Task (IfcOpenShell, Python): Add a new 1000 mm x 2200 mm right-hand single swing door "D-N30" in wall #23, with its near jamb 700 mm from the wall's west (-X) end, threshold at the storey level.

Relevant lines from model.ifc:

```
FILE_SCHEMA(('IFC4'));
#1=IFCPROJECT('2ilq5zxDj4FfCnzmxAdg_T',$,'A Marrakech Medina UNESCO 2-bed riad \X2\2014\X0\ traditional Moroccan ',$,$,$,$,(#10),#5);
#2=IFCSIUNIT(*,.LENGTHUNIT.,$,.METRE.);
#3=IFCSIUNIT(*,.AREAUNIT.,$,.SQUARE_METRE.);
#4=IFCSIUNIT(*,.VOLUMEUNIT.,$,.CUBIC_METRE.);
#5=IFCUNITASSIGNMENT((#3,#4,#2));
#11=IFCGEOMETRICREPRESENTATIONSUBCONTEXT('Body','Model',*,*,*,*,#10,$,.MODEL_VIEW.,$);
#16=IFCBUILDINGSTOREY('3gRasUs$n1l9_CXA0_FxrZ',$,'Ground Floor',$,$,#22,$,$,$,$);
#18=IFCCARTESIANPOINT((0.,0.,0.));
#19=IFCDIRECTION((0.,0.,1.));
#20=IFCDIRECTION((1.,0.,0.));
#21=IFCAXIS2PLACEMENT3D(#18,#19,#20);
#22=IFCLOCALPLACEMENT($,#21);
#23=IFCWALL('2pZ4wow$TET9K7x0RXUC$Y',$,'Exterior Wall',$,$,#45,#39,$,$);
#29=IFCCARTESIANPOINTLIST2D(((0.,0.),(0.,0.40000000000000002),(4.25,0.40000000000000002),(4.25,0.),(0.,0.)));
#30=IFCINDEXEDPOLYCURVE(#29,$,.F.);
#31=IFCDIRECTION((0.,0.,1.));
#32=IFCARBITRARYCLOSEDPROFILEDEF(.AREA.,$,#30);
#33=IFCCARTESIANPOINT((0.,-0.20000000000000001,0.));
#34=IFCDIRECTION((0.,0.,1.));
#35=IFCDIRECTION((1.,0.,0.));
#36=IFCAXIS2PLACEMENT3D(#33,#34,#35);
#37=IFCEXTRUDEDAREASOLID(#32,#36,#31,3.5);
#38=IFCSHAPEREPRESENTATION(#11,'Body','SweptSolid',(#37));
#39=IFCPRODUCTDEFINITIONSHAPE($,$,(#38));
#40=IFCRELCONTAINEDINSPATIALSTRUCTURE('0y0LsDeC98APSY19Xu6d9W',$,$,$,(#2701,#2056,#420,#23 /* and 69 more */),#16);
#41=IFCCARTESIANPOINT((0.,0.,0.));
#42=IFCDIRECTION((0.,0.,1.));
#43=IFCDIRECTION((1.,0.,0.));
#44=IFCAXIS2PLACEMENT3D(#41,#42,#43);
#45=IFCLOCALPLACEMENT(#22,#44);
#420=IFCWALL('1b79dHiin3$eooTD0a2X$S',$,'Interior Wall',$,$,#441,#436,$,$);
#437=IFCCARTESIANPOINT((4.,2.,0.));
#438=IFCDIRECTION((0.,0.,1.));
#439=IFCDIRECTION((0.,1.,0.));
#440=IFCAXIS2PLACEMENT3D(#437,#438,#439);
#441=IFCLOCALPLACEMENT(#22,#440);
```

```python
import numpy as np
import ifcopenshell
import ifcopenshell.api.feature
import ifcopenshell.api.geometry
import ifcopenshell.api.root
import ifcopenshell.api.spatial
import ifcopenshell.geom
import ifcopenshell.util.element
import ifcopenshell.util.placement
import ifcopenshell.util.representation
import ifcopenshell.util.shape
import ifcopenshell.util.unit

model = ifcopenshell.open("model.ifc")
unit_scale = ifcopenshell.util.unit.calculate_unit_scale(model)
settings = ifcopenshell.geom.settings()


def volume(element):
    """Net volume in cubic metres, openings subtracted."""
    shape = ifcopenshell.geom.create_shape(settings, element)
    return ifcopenshell.util.shape.get_volume(shape.geometry)


wall = model.by_id(23)
storey = ifcopenshell.util.element.get_container(wall, ifc_class="IfcBuildingStorey")
context = ifcopenshell.util.representation.get_context(model, "Model", "Body", "MODEL_VIEW")
before = volume(wall)

width, height, from_end, sill = 1, 2.2, 0.7, 0.0  # metres

# The wall runs along its own X axis, and the end named is its -X end.
wall_shape = ifcopenshell.geom.create_shape(settings, wall)
x, y, z = ifcopenshell.util.shape.get_vertices(wall_shape.geometry).T
start = x.min() + from_end
face, thickness = float(y.min()), float(y.max() - y.min())
wall_matrix = ifcopenshell.util.placement.get_local_placement(wall.ObjectPlacement)
level = ifcopenshell.util.placement.get_local_placement(storey.ObjectPlacement)[2, 3]


def in_wall(x, y):
    """Placement at x, y metres in the wall's axes, at sill height."""
    matrix = wall_matrix.copy()
    matrix[:, 3] = wall_matrix @ np.array([x / unit_scale, y / unit_scale, 0.0, 1.0])
    matrix[2, 3] = level + sill / unit_scale
    return matrix


# Opening: a box that overshoots both wall faces by 50 mm.
opening = ifcopenshell.api.root.create_entity(model, ifc_class="IfcOpeningElement", predefined_type="OPENING")
box = ifcopenshell.api.geometry.add_wall_representation(
    model, context=context, length=width, height=height, thickness=thickness + 0.1
)
ifcopenshell.api.geometry.assign_representation(model, product=opening, representation=box)
ifcopenshell.api.geometry.edit_object_placement(model, product=opening, matrix=in_wall(start, face - 0.05), is_si=False)
ifcopenshell.api.feature.add_feature(model, feature=opening, element=wall)

door = ifcopenshell.api.root.create_entity(model, ifc_class="IfcDoor", name="D-N30", predefined_type="DOOR")
door.OverallWidth, door.OverallHeight = width / unit_scale, height / unit_scale
door.OperationType = "SINGLE_SWING_RIGHT"
body = ifcopenshell.api.geometry.add_door_representation(
    model,
    context=context,
    overall_width=door.OverallWidth,
    overall_height=door.OverallHeight,
    operation_type="SINGLE_SWING_RIGHT",
    lining_properties={"LiningDepth": thickness / unit_scale, "ThresholdDepth": thickness / unit_scale},
)
ifcopenshell.api.geometry.assign_representation(model, product=door, representation=body)
ifcopenshell.api.spatial.assign_container(model, products=[door], relating_structure=storey)
ifcopenshell.api.feature.add_filling(model, opening=opening, element=door)

# The lining spans the wall, so the door starts at the wall face.
ifcopenshell.api.geometry.edit_object_placement(model, product=door, matrix=in_wall(start, face), is_si=False)

after = volume(wall)

print(f"wall volume {before:.3f} -> {after:.3f} m3")

model.write("model_edited.ifc")
```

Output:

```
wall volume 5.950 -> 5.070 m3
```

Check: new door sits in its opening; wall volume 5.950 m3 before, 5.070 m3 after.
